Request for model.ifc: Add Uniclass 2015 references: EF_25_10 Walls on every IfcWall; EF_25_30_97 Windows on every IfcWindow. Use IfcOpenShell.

First a look at what the model holds.

```python
import ifcopenshell

model = ifcopenshell.open("model.ifc")
print(model.schema)
print("classifications:", [c.Name for c in model.by_type("IfcClassification")])
for ifc_class in ("IfcDoor", "IfcRoof", "IfcStair", "IfcWall", "IfcWindow"):
    print(ifc_class, len(model.by_type(ifc_class)))
```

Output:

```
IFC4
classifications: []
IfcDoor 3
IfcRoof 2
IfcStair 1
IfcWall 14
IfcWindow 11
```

```python
import ifcopenshell
import ifcopenshell.api.classification

model = ifcopenshell.open("model.ifc")

system = ifcopenshell.api.classification.add_classification(model, classification="Uniclass 2015")

codes = {
    "IfcWall": ("EF_25_10", "Walls"),
    "IfcWindow": ("EF_25_30_97", "Windows"),
}
for ifc_class, (code, name) in codes.items():
    products = model.by_type(ifc_class)
    ifcopenshell.api.classification.add_reference(
        model, products=products, classification=system, identification=code, name=name
    )
    print(code, len(products))

model.write("model_edited.ifc")
```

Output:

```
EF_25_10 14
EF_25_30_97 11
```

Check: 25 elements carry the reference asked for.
